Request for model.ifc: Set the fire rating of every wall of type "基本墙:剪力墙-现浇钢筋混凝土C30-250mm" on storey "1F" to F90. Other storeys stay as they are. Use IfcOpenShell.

First a look at what the model holds.

```python
import ifcopenshell
import ifcopenshell.util.element

model = ifcopenshell.open("model.ifc")
print(model.schema)
storey = next(s for s in model.by_type("IfcBuildingStorey") if s.Name == "1F")
walls = [e for e in ifcopenshell.util.element.get_decomposition(storey) if e.is_a("IfcWall")]
seen = {}
for e in walls:
    element_type = ifcopenshell.util.element.get_type(e)
    key = (element_type.Name if element_type != e and element_type else None, ifcopenshell.util.element.get_pset(e, "Pset_WallCommon", "FireRating"))
    seen[key] = seen.get(key, 0) + 1
for (name, value), count in sorted(seen.items(), key=str):
    print(count, "x", name, "|", value)
```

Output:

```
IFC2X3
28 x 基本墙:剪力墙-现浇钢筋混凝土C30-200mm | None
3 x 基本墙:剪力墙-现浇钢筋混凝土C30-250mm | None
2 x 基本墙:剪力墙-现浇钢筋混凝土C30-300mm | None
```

```python
import ifcopenshell
import ifcopenshell.api.pset
import ifcopenshell.util.element

model = ifcopenshell.open("model.ifc")

storey = next(s for s in model.by_type("IfcBuildingStorey") if s.Name == "1F")
walls = [e for e in ifcopenshell.util.element.get_decomposition(storey) if e.is_a("IfcWall")]

count = 0
for e in walls:
    element_type = ifcopenshell.util.element.get_type(e)
    if element_type in (None, e) or element_type.Name != "基本墙:剪力墙-现浇钢筋混凝土C30-250mm":
        continue
    # add_pset returns the element's existing set when there is one.
    pset = ifcopenshell.api.pset.add_pset(model, product=e, name="Pset_WallCommon")
    ifcopenshell.api.pset.edit_pset(model, pset=pset, properties={"FireRating": "F90"})
    count += 1

print(count, "walls updated")

model.write("model-out.ifc")
```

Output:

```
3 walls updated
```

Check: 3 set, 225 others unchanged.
